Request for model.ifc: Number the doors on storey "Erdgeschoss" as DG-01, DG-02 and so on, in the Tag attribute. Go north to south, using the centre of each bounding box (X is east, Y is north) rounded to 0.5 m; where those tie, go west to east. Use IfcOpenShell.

First a look at what the model holds.

```python
import ifcopenshell
import ifcopenshell.util.element
import ifcopenshell.util.placement

model = ifcopenshell.open("model.ifc")
print(model.schema)
storey = next(s for s in model.by_type("IfcBuildingStorey") if s.Name == "Erdgeschoss")
doors = [e for e in ifcopenshell.util.element.get_decomposition(storey) if e.is_a("IfcDoor")]
for e in sorted(doors, key=lambda e: e.id()):
    origin = ifcopenshell.util.placement.get_local_placement(e.ObjectPlacement)[:3, 3]
    print(e.id(), e.Tag, e.Name, origin.round(2) + 0.0, sep=" | ")
```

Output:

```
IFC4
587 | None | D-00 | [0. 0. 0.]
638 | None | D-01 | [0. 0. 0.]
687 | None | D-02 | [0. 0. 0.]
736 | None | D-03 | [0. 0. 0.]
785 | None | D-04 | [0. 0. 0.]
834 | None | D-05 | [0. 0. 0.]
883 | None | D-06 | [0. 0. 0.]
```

```python
import ifcopenshell
import ifcopenshell.geom
import ifcopenshell.util.element
import ifcopenshell.util.shape

model = ifcopenshell.open("model.ifc")
settings = ifcopenshell.geom.settings()
settings.set("use-world-coords", True)


def centre(element):
    shape = ifcopenshell.geom.create_shape(settings, element)
    return ifcopenshell.util.shape.get_bbox_centroid(shape.geometry)


storey = next(s for s in model.by_type("IfcBuildingStorey") if s.Name == "Erdgeschoss")
doors = [e for e in ifcopenshell.util.element.get_decomposition(storey) if e.is_a("IfcDoor")]

# Insertion points can sit at a corner or the storey origin, so sort by the geometry (in metres).
centres = {e: centre(e) for e in doors}
doors.sort(key=lambda e: (-round(centres[e][1] / 0.5), centres[e][0]))

for i, e in enumerate(doors, start=1):
    number = f"DG-{i:02d}"
    e.Tag = number
    print(e.id(), number)

model.write("model_edited.ifc")
```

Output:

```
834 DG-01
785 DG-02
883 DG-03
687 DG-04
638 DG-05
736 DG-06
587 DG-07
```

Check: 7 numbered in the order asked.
